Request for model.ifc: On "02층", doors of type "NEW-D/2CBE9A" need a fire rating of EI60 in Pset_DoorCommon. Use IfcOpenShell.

First a look at what the model holds.

```python
import ifcopenshell
import ifcopenshell.util.element

model = ifcopenshell.open("model.ifc")
print(model.schema)
storey = next(s for s in model.by_type("IfcBuildingStorey") if s.Name == "02층")
doors = [e for e in ifcopenshell.util.element.get_decomposition(storey) if e.is_a("IfcDoor")]
seen = {}
for e in doors:
    element_type = ifcopenshell.util.element.get_type(e)
    key = (element_type.Name if element_type != e and element_type else None, ifcopenshell.util.element.get_pset(e, "Pset_DoorCommon", "FireRating"))
    seen[key] = seen.get(key, 0) + 1
for (name, value), count in sorted(seen.items(), key=str):
    print(count, "x", name, "|", value)
```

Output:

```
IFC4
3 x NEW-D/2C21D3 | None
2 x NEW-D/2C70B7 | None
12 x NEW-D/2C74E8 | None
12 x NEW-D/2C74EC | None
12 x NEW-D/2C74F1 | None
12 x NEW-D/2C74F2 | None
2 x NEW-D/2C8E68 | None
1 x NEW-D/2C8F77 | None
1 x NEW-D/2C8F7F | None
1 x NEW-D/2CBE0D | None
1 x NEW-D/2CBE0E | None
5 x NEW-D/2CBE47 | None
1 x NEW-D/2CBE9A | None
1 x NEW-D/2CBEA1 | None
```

```python
import ifcopenshell
import ifcopenshell.api.pset
import ifcopenshell.util.element

model = ifcopenshell.open("model.ifc")

storey = next(s for s in model.by_type("IfcBuildingStorey") if s.Name == "02층")
doors = [e for e in ifcopenshell.util.element.get_decomposition(storey) if e.is_a("IfcDoor")]

count = 0
for e in doors:
    element_type = ifcopenshell.util.element.get_type(e)
    if element_type in (None, e) or element_type.Name != "NEW-D/2CBE9A":
        continue
    # add_pset returns the element's existing set when there is one.
    pset = ifcopenshell.api.pset.add_pset(model, product=e, name="Pset_DoorCommon")
    ifcopenshell.api.pset.edit_pset(model, pset=pset, properties={"FireRating": "EI60"})
    count += 1

print(count, "doors updated")

model.write("model_edited.ifc")
```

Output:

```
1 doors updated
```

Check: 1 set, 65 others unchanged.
